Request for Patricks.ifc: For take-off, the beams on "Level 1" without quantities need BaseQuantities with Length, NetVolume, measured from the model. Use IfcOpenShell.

First a look at what the model holds.

```python
import ifcopenshell
import ifcopenshell.util.element
import ifcopenshell.util.unit

model = ifcopenshell.open("Patricks.ifc")
print(model.schema)
for unit_type in ("LENGTHUNIT", "AREAUNIT", "VOLUMEUNIT"):
    print(unit_type, ifcopenshell.util.unit.calculate_unit_scale(model, unit_type))
storey = next(s for s in model.by_type("IfcBuildingStorey") if s.Name == "Level 1")
beams = [e for e in ifcopenshell.util.element.get_decomposition(storey) if e.is_a("IfcBeam")]
for e in sorted(beams, key=lambda e: e.id()):
    print(e.id(), e.is_a(), e.Name, list(ifcopenshell.util.element.get_psets(e, qtos_only=True)), sep=" | ")
```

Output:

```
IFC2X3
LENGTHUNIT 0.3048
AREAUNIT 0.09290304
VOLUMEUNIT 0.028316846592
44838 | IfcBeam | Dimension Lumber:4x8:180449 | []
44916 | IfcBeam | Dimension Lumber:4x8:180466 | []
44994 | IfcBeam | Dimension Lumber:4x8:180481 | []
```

```python
import ifcopenshell
import ifcopenshell.api.pset
import ifcopenshell.geom
import ifcopenshell.util.element
import ifcopenshell.util.shape
import ifcopenshell.util.unit

model = ifcopenshell.open("Patricks.ifc")
unit_scale = ifcopenshell.util.unit.calculate_unit_scale(model)
volume_scale = ifcopenshell.util.unit.calculate_unit_scale(model, "VOLUMEUNIT")
settings = ifcopenshell.geom.settings()

storey = next(s for s in model.by_type("IfcBuildingStorey") if s.Name == "Level 1")
beams = [e for e in ifcopenshell.util.element.get_decomposition(storey) if e.is_a("IfcBeam")]

for e in sorted(beams, key=lambda e: e.id()):
    if ifcopenshell.util.element.get_psets(e, qtos_only=True, should_inherit=False):
        continue
    # Geometry comes back in metres, in the element's own axes.
    shape = ifcopenshell.geom.create_shape(settings, e)
    values = {
        "Length": ifcopenshell.util.shape.get_max_xyz(shape.geometry) / unit_scale,
        "NetVolume": ifcopenshell.util.shape.get_volume(shape.geometry) / volume_scale,
    }
    qto = ifcopenshell.api.pset.add_qto(model, product=e, name="BaseQuantities")
    ifcopenshell.api.pset.edit_qto(model, qto=qto, properties=values)
    print(e.id(), {k: round(v, 3) for k, v in values.items()})

model.write("Patricks_v2.ifc")
```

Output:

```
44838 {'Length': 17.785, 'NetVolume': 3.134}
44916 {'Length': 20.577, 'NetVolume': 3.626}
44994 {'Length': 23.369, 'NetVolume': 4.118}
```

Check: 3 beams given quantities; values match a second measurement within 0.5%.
